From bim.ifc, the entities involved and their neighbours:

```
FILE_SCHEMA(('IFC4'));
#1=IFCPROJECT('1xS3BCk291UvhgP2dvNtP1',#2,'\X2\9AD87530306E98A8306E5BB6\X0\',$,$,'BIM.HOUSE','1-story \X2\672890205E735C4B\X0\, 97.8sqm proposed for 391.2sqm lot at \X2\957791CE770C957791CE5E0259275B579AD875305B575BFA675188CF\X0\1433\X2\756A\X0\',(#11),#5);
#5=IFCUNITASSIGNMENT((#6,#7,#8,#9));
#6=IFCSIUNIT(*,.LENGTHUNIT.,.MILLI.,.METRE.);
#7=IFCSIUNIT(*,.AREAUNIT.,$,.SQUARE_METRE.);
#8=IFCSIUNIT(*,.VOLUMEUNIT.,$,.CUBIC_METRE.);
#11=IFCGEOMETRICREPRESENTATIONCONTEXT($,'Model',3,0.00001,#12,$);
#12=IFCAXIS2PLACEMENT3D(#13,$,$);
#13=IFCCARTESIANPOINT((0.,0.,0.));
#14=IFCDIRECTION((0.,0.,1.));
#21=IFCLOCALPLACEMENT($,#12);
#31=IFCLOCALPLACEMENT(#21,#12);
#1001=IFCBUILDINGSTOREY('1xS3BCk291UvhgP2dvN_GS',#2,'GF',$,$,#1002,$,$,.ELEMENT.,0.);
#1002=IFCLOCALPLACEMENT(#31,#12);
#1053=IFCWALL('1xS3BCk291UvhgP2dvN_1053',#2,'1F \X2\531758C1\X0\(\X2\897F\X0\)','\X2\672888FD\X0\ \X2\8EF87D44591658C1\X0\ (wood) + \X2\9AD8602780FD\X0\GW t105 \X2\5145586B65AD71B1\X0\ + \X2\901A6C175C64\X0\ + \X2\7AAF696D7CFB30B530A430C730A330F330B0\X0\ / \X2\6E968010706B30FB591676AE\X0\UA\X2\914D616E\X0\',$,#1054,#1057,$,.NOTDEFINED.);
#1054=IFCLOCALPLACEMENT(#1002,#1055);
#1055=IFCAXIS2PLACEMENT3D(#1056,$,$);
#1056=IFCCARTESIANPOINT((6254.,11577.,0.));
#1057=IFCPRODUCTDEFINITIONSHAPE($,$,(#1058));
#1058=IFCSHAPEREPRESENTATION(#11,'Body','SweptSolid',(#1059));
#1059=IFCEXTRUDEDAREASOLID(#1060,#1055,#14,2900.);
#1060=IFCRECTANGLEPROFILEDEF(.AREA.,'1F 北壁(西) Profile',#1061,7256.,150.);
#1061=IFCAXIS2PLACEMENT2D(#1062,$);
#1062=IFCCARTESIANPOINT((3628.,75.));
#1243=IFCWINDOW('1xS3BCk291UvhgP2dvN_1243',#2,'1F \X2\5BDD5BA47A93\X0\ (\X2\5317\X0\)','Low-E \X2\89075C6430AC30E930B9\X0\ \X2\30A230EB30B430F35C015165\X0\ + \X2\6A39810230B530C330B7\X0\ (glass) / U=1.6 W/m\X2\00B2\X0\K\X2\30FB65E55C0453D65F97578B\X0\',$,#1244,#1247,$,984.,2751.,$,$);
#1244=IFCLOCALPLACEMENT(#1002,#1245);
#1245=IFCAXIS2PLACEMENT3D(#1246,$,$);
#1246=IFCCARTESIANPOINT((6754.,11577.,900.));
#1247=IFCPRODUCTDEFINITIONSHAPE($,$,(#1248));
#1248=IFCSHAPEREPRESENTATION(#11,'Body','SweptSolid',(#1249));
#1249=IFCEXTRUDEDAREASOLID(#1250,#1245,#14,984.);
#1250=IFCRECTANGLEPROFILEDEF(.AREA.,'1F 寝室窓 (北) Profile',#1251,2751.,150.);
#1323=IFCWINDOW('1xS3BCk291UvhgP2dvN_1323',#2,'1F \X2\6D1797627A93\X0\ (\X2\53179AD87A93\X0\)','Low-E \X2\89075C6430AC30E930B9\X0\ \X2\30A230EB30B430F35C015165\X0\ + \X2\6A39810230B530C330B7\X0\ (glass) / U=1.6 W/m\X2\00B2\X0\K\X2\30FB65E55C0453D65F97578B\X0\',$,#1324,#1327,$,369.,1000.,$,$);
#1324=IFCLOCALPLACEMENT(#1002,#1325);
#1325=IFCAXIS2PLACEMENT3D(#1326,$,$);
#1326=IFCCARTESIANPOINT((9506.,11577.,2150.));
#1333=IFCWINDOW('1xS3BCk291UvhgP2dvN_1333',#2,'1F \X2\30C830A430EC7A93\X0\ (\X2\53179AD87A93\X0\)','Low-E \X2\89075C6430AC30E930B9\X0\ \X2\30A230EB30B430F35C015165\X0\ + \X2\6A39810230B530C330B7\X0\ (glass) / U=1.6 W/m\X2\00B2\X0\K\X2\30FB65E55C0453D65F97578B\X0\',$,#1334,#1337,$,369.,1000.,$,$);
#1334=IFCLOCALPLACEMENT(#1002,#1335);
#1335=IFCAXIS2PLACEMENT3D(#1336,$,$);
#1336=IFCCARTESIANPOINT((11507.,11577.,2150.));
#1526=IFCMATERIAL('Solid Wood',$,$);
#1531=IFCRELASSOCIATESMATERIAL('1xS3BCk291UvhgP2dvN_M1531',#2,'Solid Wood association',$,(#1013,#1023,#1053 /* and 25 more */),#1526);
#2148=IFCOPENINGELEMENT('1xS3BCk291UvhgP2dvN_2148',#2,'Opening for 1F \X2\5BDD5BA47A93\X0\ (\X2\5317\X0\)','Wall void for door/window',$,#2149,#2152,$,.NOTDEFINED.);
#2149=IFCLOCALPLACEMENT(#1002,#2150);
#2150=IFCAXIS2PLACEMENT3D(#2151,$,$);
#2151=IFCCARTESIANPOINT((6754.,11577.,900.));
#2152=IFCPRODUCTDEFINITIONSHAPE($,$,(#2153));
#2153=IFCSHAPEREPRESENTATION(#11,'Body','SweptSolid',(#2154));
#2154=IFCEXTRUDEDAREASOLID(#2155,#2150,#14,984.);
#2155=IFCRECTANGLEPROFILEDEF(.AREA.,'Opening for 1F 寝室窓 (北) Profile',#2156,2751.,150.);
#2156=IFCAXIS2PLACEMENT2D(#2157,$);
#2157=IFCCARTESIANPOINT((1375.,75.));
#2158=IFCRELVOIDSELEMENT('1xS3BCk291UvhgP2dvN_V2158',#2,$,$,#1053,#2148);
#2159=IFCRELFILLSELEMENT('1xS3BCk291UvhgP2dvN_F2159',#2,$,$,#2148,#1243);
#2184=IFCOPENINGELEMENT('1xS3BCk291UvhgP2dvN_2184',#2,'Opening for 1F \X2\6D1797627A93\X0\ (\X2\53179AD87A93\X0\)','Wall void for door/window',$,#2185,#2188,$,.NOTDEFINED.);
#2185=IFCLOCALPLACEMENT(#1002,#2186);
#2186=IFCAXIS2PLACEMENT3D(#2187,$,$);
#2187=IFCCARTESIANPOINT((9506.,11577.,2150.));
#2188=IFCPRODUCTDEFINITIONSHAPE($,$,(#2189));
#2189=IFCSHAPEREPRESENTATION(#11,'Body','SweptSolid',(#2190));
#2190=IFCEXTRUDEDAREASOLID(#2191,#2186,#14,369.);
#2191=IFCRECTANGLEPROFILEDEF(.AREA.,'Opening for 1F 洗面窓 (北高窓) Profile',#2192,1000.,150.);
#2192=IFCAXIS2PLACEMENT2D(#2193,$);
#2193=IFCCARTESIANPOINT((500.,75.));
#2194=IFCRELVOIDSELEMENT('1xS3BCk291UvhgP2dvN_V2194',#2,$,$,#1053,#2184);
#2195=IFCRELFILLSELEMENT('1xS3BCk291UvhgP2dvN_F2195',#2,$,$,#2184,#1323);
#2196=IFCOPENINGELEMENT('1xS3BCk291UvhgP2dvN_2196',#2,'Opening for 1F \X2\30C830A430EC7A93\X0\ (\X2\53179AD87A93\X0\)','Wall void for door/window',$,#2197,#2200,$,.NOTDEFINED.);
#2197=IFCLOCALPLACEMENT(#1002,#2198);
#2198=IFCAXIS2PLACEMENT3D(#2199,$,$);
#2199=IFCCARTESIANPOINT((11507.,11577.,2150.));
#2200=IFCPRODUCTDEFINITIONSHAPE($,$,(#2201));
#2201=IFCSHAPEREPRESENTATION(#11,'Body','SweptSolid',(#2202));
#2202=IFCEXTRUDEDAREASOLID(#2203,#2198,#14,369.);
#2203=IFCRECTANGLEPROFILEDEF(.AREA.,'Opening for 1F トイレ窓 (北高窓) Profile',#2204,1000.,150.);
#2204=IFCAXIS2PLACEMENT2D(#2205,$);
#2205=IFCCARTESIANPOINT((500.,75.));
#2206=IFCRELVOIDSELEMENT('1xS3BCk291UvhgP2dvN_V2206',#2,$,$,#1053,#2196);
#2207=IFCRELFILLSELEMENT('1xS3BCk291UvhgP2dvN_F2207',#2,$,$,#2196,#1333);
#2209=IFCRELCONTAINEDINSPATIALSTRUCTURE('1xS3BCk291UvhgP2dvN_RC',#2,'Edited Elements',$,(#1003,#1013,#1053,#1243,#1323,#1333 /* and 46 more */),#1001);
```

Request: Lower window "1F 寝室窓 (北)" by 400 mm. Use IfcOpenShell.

```python
import numpy as np
import ifcopenshell
import ifcopenshell.api.geometry
import ifcopenshell.util.placement
import ifcopenshell.util.unit

model = ifcopenshell.open("bim.ifc")
unit_scale = ifcopenshell.util.unit.calculate_unit_scale(model)

window = model.by_guid("1xS3BCk291UvhgP2dvN_1243")
opening = window.FillsVoids[0].RelatingOpeningElement
dz = -0.4 / unit_scale

shift = np.array([0.0, 0.0, dz])
# The window is not placed relative to its opening, so move both.
for product in (opening, window):
    matrix = ifcopenshell.util.placement.get_local_placement(product.ObjectPlacement)
    matrix[:3, 3] += shift
    ifcopenshell.api.geometry.edit_object_placement(model, product=product, matrix=matrix, is_si=False)

print(f"moved by {dz * unit_scale:+.3f} m")

model.write("bim_edited.ifc")
```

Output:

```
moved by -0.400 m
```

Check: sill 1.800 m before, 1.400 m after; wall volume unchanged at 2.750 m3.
